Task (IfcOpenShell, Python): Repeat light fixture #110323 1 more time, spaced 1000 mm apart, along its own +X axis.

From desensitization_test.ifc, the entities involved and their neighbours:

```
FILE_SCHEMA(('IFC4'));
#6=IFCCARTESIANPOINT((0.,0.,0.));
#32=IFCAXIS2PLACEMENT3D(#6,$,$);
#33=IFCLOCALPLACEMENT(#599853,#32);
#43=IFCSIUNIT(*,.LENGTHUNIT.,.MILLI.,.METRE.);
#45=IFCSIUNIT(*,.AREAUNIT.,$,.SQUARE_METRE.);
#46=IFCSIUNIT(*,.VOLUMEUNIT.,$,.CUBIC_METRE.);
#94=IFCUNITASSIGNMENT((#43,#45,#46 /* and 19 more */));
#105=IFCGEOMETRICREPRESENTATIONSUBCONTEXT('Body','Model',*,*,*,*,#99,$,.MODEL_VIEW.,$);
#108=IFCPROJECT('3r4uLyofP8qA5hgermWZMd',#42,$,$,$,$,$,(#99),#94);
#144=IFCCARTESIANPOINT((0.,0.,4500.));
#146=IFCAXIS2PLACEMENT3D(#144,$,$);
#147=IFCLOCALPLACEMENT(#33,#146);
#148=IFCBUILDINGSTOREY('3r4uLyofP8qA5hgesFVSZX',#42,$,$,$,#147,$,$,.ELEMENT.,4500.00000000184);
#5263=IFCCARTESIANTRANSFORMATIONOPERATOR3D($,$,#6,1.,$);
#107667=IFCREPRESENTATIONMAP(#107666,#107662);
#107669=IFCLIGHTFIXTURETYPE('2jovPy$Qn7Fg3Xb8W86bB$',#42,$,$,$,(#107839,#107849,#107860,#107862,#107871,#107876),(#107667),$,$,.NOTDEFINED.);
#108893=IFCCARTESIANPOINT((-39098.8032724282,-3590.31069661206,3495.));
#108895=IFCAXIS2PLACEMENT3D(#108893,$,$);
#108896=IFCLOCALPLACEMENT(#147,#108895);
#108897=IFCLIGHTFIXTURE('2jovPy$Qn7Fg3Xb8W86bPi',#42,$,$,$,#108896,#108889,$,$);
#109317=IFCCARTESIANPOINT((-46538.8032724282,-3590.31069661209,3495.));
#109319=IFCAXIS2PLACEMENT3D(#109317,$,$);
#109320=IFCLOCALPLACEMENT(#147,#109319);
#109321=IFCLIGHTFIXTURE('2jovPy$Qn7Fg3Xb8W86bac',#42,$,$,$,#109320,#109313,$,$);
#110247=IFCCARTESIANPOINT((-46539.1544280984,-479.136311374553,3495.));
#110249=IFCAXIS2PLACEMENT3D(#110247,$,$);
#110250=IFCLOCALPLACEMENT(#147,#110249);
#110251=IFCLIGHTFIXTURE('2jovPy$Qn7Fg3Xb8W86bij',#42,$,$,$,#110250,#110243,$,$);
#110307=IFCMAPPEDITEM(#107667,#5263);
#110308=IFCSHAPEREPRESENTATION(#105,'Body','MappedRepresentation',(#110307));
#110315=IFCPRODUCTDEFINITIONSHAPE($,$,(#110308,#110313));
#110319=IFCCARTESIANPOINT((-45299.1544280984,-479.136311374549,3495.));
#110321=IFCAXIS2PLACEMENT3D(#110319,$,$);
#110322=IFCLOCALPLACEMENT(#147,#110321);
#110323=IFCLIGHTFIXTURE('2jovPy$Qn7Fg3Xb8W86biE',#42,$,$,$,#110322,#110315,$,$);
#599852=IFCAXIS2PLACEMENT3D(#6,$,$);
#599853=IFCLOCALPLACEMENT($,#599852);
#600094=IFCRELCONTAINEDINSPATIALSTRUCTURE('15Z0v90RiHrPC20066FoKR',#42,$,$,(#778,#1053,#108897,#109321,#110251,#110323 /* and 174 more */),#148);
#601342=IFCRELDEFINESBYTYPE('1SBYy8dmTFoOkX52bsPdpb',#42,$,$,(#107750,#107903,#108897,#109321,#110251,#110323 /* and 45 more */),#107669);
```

```python
import ifcopenshell
import ifcopenshell.api.geometry
import ifcopenshell.api.root
import ifcopenshell.util.element
import ifcopenshell.util.placement

model = ifcopenshell.open("desensitization_test.ifc")


def reuse_history(source, copy):
    """copy_class also copies each property set's owner history, people and application; keep the originals."""
    for rel in copy.IsDefinedBy:
        if rel.is_a("IfcRelDefinesByProperties") and (history := rel.RelatingPropertyDefinition.OwnerHistory):
            rel.RelatingPropertyDefinition.OwnerHistory = source.OwnerHistory
            ifcopenshell.util.element.remove_deep2(model, history)


source = model.by_guid("2jovPy$Qn7Fg3Xb8W86biE")
base = ifcopenshell.util.placement.get_local_placement(source.ObjectPlacement)
step = base[:3, 0] * 1000.0

for i in range(1, 2):
    copy = ifcopenshell.api.root.copy_class(model, product=source)
    copy.Representation = ifcopenshell.util.element.copy_deep(
        model, source.Representation, exclude=["IfcGeometricRepresentationContext", "IfcRepresentationMap"]
    )
    reuse_history(source, copy)
    matrix = base.copy()
    matrix[:3, 3] += i * step
    print("added at", matrix[:3, 3].round(3) + 0.0)
    ifcopenshell.api.geometry.edit_object_placement(model, product=copy, matrix=matrix, is_si=False)

model.write("desensitization_test-out.ifc")
```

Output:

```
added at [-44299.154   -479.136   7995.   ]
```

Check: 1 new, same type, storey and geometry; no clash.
